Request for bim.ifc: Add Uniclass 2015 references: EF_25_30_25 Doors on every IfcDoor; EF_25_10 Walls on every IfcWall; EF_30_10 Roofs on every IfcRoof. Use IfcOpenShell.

First a look at what the model holds.

```python
import ifcopenshell

model = ifcopenshell.open("bim.ifc")
print(model.schema)
print("classifications:", [c.Name for c in model.by_type("IfcClassification")])
for ifc_class in ("IfcDoor", "IfcRoof", "IfcStair", "IfcWall", "IfcWindow"):
    print(ifc_class, len(model.by_type(ifc_class)))
```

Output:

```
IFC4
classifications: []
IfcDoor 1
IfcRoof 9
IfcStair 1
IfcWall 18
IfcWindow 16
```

```python
import ifcopenshell
import ifcopenshell.api.classification

model = ifcopenshell.open("bim.ifc")

system = ifcopenshell.api.classification.add_classification(model, classification="Uniclass 2015")

codes = {
    "IfcDoor": ("EF_25_30_25", "Doors"),
    "IfcWall": ("EF_25_10", "Walls"),
    "IfcRoof": ("EF_30_10", "Roofs"),
}
for ifc_class, (code, name) in codes.items():
    products = model.by_type(ifc_class)
    ifcopenshell.api.classification.add_reference(
        model, products=products, classification=system, identification=code, name=name
    )
    print(code, len(products))

model.write("bim_edited.ifc")
```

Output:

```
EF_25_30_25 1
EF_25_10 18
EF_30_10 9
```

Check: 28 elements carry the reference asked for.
